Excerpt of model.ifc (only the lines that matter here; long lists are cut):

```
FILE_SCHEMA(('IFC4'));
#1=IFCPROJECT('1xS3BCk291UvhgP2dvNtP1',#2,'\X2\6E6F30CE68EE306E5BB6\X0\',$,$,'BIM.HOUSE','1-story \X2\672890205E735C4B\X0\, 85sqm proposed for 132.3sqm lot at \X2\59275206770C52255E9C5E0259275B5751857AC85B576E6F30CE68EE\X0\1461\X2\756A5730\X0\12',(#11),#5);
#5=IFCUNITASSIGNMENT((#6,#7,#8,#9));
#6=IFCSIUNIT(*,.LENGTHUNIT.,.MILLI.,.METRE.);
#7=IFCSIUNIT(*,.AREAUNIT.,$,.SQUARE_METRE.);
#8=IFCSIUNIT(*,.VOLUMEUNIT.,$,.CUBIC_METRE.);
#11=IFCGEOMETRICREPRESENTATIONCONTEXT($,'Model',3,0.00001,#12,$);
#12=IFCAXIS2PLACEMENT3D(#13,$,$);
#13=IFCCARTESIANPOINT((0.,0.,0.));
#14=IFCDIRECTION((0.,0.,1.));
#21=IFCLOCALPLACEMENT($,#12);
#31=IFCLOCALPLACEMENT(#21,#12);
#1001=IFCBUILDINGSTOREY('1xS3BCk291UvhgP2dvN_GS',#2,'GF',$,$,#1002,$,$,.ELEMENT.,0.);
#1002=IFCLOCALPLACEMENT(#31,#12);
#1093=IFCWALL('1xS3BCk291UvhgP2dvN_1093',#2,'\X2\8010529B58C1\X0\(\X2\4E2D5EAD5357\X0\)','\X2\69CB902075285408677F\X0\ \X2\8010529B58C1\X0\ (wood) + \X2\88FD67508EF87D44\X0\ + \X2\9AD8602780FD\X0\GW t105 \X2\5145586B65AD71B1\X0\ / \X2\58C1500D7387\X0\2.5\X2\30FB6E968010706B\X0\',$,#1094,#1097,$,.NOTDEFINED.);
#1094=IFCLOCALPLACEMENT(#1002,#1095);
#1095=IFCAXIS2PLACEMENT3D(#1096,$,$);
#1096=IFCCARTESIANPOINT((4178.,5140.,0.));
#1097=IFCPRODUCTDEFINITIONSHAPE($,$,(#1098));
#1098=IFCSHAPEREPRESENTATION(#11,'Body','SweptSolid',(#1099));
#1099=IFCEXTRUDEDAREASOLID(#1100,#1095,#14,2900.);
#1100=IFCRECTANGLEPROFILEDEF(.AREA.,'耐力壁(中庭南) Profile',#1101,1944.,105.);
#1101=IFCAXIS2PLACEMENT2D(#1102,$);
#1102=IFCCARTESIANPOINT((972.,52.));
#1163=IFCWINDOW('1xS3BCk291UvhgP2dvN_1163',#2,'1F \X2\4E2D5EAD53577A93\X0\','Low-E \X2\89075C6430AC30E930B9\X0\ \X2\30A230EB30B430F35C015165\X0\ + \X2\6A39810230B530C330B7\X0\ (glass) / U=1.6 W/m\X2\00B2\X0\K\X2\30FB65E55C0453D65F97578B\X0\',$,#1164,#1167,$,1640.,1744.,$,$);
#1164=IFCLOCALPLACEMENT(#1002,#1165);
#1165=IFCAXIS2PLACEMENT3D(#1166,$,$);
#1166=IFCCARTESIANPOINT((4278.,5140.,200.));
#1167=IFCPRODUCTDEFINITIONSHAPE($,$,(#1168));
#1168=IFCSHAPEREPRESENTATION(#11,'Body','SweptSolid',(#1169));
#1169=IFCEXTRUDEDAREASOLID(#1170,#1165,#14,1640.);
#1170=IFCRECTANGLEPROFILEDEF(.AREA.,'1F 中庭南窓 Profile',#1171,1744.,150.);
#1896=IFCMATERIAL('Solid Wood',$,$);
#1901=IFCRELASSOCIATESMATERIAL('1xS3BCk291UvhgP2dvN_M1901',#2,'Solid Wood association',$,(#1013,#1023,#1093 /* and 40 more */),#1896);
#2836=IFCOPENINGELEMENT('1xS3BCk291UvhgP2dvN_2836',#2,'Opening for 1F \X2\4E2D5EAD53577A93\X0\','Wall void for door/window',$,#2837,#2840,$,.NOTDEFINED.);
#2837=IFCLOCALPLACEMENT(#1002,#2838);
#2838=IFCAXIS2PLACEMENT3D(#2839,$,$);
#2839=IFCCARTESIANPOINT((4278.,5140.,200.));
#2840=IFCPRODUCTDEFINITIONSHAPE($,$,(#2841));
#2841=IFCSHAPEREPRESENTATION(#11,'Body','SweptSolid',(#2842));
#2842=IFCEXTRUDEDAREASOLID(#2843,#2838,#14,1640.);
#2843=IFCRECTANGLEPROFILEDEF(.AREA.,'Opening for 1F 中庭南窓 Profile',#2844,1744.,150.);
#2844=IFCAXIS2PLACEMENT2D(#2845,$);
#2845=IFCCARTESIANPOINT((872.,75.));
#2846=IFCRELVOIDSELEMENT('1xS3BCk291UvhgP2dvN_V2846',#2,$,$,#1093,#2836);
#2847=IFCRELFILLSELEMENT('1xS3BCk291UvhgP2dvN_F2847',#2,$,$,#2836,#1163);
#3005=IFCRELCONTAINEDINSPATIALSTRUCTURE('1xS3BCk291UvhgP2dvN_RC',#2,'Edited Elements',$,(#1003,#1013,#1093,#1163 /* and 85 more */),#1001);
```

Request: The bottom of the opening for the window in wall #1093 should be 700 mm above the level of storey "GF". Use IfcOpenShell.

```python
import numpy as np
import ifcopenshell
import ifcopenshell.api.geometry
import ifcopenshell.geom
import ifcopenshell.util.element
import ifcopenshell.util.placement
import ifcopenshell.util.shape
import ifcopenshell.util.unit

model = ifcopenshell.open("model.ifc")
unit_scale = ifcopenshell.util.unit.calculate_unit_scale(model)

window = model.by_guid("1xS3BCk291UvhgP2dvN_1163")
opening = window.FillsVoids[0].RelatingOpeningElement
storey = ifcopenshell.util.element.get_container(window, ifc_class="IfcBuildingStorey")
level = ifcopenshell.util.placement.get_local_placement(storey.ObjectPlacement)[2, 3]

# The opening's origin need not be at the sill, so measure its lowest point.
shape = ifcopenshell.geom.create_shape(ifcopenshell.geom.settings(), opening)
bottom = ifcopenshell.util.shape.get_shape_bottom_elevation(shape, shape.geometry) / unit_scale
dz = level + 700.0 - bottom

shift = np.array([0.0, 0.0, dz])
# The window is not placed relative to its opening, so move both.
for product in (opening, window):
    matrix = ifcopenshell.util.placement.get_local_placement(product.ObjectPlacement)
    matrix[:3, 3] += shift
    ifcopenshell.api.geometry.edit_object_placement(model, product=product, matrix=matrix, is_si=False)

print(f"moved by {dz * unit_scale:+.3f} m")

model.write("model-out.ifc")
```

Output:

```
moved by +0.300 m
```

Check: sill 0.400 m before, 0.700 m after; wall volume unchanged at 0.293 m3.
